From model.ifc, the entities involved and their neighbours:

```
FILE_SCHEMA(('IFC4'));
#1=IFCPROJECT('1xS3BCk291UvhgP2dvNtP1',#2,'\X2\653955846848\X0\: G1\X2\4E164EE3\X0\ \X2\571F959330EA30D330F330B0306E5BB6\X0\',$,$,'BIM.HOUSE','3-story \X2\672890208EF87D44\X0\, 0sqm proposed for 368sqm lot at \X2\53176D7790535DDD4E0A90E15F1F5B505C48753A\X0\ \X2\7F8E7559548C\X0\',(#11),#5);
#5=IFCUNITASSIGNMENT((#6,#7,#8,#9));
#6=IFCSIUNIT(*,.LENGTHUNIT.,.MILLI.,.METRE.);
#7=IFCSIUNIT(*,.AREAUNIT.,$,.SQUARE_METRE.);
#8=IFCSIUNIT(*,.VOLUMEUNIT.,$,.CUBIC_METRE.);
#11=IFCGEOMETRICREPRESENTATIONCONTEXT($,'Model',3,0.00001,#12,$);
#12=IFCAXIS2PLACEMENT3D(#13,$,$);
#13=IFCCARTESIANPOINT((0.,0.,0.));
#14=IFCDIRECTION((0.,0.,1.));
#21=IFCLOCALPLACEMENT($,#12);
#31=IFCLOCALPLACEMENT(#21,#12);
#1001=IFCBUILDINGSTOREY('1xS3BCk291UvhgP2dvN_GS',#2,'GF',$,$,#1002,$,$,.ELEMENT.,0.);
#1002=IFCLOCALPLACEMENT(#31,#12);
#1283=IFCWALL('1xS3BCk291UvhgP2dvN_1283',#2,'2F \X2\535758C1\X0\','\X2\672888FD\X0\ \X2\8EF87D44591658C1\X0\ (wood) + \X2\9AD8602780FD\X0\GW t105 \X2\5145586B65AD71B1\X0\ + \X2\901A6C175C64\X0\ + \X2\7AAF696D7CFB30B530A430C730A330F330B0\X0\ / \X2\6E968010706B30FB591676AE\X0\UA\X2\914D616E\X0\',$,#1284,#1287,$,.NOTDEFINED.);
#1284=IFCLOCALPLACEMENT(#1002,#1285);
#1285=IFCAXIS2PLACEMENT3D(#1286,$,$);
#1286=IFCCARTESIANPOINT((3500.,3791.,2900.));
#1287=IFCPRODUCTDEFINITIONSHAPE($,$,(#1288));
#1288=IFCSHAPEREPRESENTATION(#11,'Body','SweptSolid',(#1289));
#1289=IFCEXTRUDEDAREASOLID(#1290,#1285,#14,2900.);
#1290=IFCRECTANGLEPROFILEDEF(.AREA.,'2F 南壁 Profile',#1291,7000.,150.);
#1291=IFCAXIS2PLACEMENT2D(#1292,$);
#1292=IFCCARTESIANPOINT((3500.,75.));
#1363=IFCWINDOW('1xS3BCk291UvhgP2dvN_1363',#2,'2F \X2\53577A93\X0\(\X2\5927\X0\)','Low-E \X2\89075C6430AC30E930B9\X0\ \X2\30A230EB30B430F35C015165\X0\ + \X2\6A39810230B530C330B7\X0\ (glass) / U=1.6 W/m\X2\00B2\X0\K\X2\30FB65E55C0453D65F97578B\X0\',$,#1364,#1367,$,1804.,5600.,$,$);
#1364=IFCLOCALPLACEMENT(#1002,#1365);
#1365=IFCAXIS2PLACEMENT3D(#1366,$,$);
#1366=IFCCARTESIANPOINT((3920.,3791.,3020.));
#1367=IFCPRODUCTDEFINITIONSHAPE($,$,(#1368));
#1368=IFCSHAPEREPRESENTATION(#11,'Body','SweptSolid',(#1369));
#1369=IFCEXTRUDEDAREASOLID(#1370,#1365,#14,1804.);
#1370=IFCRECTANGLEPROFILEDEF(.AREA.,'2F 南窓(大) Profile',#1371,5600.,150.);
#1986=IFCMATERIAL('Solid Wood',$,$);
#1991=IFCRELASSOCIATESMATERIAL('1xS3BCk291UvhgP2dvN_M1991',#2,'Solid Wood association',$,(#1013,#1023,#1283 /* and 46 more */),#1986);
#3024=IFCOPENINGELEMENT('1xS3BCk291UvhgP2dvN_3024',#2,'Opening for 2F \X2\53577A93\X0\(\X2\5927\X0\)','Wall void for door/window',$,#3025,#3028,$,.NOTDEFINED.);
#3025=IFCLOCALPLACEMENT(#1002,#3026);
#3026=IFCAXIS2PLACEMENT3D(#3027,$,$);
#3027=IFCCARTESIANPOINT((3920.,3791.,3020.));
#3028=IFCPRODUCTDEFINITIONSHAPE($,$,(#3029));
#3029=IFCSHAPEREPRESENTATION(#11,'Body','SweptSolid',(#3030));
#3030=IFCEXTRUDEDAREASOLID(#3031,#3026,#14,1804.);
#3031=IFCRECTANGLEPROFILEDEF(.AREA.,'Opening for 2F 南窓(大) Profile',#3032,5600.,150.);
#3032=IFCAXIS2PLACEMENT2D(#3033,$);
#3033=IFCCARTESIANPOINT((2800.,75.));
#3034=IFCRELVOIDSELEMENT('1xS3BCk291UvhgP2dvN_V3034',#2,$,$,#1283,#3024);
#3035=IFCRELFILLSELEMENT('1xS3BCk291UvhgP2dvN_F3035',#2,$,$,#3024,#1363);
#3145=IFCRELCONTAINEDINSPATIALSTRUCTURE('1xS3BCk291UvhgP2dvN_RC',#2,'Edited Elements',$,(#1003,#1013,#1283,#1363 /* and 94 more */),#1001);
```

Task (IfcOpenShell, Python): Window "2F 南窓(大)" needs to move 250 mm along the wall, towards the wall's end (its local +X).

```python
import ifcopenshell
import ifcopenshell.api.geometry
import ifcopenshell.util.placement
import ifcopenshell.util.unit

model = ifcopenshell.open("model.ifc")
unit_scale = ifcopenshell.util.unit.calculate_unit_scale(model)

window = model.by_id(1363)
opening = window.FillsVoids[0].RelatingOpeningElement
wall = opening.VoidsElements[0].RelatingBuildingElement

wall_matrix = ifcopenshell.util.placement.get_local_placement(wall.ObjectPlacement)
shift = wall_matrix[:3, 0] * 0.25 / unit_scale
before = ifcopenshell.util.placement.get_local_placement(window.ObjectPlacement)[:3, 3].copy()

# The window is not placed relative to its opening, so move both.
for product in (opening, window):
    matrix = ifcopenshell.util.placement.get_local_placement(product.ObjectPlacement)
    matrix[:3, 3] += shift
    ifcopenshell.api.geometry.edit_object_placement(model, product=product, matrix=matrix, is_si=False)

after = ifcopenshell.util.placement.get_local_placement(window.ObjectPlacement)[:3, 3]
print("window moved by", (after - before).round(3) + 0.0)

model.write("model_edited.ifc")
```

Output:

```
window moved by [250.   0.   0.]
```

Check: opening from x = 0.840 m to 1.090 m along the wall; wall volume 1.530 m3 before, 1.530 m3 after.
